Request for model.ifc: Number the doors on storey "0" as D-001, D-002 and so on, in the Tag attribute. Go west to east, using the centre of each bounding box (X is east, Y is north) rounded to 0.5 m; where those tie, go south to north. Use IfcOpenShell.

First a look at what the model holds.

```python
import ifcopenshell
import ifcopenshell.util.element
import ifcopenshell.util.placement

model = ifcopenshell.open("model.ifc")
print(model.schema)
storey = next(s for s in model.by_type("IfcBuildingStorey") if s.Name == "0")
doors = [e for e in ifcopenshell.util.element.get_decomposition(storey) if e.is_a("IfcDoor")]
for e in sorted(doors, key=lambda e: e.id()):
    origin = ifcopenshell.util.placement.get_local_placement(e.ObjectPlacement)[:3, 3]
    print(e.id(), e.Tag, e.Name, origin.round(2) + 0.0, sep=" | ")
```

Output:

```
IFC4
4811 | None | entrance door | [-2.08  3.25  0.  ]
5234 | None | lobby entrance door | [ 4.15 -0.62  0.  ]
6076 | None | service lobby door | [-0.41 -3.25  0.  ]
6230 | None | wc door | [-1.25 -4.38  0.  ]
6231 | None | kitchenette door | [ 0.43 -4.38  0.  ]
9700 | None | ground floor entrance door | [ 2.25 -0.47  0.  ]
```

```python
import ifcopenshell
import ifcopenshell.geom
import ifcopenshell.util.element
import ifcopenshell.util.shape

model = ifcopenshell.open("model.ifc")
settings = ifcopenshell.geom.settings()
settings.set("use-world-coords", True)


def centre(element):
    shape = ifcopenshell.geom.create_shape(settings, element)
    return ifcopenshell.util.shape.get_bbox_centroid(shape.geometry)


storey = next(s for s in model.by_type("IfcBuildingStorey") if s.Name == "0")
doors = [e for e in ifcopenshell.util.element.get_decomposition(storey) if e.is_a("IfcDoor")]

# Insertion points can sit at a corner or the storey origin, so sort by the geometry (in metres).
centres = {e: centre(e) for e in doors}
doors.sort(key=lambda e: (round(centres[e][0] / 0.5), centres[e][1]))

for i, e in enumerate(doors, start=1):
    number = f"D-0{i:02d}"
    e.Tag = number
    print(e.id(), number)

model.write("model_edited.ifc")
```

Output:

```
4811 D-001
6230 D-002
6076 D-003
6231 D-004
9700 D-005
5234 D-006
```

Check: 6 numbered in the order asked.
